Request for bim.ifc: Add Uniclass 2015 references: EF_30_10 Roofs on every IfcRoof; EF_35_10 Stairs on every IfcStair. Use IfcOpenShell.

First a look at what the model holds.

```python
import ifcopenshell

model = ifcopenshell.open("bim.ifc")
print(model.schema)
print("classifications:", [c.Name for c in model.by_type("IfcClassification")])
for ifc_class in ("IfcDoor", "IfcRoof", "IfcStair", "IfcWall", "IfcWindow"):
    print(ifc_class, len(model.by_type(ifc_class)))
```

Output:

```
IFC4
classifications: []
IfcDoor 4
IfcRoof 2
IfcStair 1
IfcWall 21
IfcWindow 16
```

```python
import ifcopenshell
import ifcopenshell.api.classification

model = ifcopenshell.open("bim.ifc")

system = ifcopenshell.api.classification.add_classification(model, classification="Uniclass 2015")

codes = {
    "IfcRoof": ("EF_30_10", "Roofs"),
    "IfcStair": ("EF_35_10", "Stairs"),
}
for ifc_class, (code, name) in codes.items():
    products = model.by_type(ifc_class)
    ifcopenshell.api.classification.add_reference(
        model, products=products, classification=system, identification=code, name=name
    )
    print(code, len(products))

model.write("bim_rev.ifc")
```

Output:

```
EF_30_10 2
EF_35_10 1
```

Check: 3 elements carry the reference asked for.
